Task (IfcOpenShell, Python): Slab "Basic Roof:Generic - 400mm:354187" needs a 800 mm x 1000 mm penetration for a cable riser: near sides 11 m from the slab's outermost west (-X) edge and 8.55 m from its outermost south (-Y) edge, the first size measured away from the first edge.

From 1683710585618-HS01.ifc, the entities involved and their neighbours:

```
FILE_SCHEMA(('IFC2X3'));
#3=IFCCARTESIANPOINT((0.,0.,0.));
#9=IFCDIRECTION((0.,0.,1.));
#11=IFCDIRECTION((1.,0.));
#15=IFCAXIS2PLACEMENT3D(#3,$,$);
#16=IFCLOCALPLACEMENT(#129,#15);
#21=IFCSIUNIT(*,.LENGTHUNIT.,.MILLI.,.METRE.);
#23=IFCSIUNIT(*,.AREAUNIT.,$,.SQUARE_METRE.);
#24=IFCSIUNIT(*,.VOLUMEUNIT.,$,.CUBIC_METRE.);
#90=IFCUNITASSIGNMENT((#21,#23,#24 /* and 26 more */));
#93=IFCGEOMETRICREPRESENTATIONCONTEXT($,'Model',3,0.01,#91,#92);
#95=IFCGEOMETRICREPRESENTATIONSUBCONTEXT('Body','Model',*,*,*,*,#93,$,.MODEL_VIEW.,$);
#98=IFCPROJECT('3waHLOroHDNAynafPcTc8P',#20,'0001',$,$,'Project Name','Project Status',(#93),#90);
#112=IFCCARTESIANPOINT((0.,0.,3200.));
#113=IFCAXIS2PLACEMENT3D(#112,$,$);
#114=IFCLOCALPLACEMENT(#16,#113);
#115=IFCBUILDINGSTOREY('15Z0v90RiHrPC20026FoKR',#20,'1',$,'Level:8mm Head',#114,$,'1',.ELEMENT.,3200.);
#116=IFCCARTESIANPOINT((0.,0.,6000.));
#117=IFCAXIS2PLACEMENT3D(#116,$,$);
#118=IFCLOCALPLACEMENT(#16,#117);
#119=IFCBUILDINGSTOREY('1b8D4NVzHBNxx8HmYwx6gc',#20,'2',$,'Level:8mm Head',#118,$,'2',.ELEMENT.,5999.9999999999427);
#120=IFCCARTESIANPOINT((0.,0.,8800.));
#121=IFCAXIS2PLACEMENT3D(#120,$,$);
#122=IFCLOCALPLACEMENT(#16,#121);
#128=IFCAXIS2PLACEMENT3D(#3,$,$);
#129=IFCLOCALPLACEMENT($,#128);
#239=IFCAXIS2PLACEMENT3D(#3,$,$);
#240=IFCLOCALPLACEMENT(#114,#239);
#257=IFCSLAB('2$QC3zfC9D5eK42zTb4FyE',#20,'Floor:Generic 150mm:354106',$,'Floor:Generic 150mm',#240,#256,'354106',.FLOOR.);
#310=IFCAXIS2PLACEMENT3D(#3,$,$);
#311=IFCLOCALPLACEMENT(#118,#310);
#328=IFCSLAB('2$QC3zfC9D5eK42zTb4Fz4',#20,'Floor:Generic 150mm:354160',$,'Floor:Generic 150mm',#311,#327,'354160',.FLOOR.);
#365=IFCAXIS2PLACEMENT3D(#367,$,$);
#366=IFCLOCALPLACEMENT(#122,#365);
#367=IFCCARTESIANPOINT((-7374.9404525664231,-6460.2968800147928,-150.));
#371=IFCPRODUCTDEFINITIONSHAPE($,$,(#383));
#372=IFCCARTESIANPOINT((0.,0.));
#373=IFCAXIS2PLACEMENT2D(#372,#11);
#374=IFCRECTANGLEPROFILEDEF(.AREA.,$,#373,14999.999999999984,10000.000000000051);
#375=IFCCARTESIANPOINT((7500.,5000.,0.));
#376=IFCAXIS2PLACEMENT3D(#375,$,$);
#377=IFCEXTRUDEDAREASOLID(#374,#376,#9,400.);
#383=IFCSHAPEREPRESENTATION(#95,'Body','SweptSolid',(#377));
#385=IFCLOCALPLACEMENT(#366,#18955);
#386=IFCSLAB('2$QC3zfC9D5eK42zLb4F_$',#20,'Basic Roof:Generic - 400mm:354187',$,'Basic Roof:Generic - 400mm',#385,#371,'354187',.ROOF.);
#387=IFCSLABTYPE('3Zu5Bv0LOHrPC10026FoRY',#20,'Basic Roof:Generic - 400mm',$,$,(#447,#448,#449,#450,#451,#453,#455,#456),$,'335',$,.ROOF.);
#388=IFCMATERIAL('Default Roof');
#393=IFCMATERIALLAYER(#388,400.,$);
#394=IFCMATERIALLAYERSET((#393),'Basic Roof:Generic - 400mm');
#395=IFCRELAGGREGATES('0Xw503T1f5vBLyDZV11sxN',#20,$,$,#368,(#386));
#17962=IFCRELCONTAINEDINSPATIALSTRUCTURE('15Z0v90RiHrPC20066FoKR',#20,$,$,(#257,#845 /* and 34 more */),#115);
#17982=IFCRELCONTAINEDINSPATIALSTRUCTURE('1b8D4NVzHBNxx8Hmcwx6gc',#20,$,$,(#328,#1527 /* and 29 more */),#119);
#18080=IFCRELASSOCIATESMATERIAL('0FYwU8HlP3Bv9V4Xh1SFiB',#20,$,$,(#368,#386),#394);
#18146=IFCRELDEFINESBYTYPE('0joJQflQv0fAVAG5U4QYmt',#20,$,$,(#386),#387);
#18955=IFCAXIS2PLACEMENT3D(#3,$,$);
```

```python
import numpy as np
import ifcopenshell
import ifcopenshell.api.feature
import ifcopenshell.api.geometry
import ifcopenshell.api.root
import ifcopenshell.geom
import ifcopenshell.util.placement
import ifcopenshell.util.representation
import ifcopenshell.util.shape
import ifcopenshell.util.unit

model = ifcopenshell.open("1683710585618-HS01.ifc")
unit_scale = ifcopenshell.util.unit.calculate_unit_scale(model)
settings = ifcopenshell.geom.settings()


def volume(element):
    """Net volume in cubic metres, openings subtracted."""
    shape = ifcopenshell.geom.create_shape(settings, element)
    return ifcopenshell.util.shape.get_volume(shape.geometry)


slab = model.by_id(386)
before = volume(slab)

# Extent in the slab's own axes, in metres. The edges named are its -X and -Y sides.
slab_shape = ifcopenshell.geom.create_shape(settings, slab)
vertices = ifcopenshell.util.shape.get_vertices(slab_shape.geometry)
x_min, y_min, bottom = vertices.min(axis=0)
top = vertices[:, 2].max()

opening = ifcopenshell.api.root.create_entity(model, ifc_class="IfcOpeningElement", name="Cable riser opening")
context = ifcopenshell.util.representation.get_context(model, "Model", "Body", "MODEL_VIEW")
width, depth = 0.8, 1
outline = [(0.0, 0.0), (width, 0.0), (width, depth), (0.0, depth), (0.0, 0.0)]
# Overshoot both faces by 50 mm so the cut is clean.
shape = ifcopenshell.api.geometry.add_slab_representation(
    model, context=context, depth=top - bottom + 0.1, polyline=outline
)
ifcopenshell.api.geometry.assign_representation(model, product=opening, representation=shape)

matrix = ifcopenshell.util.placement.get_local_placement(slab.ObjectPlacement)
matrix[:, 3] = matrix @ np.append(np.array([x_min + 11, y_min + 8.55, bottom - 0.05]) / unit_scale, 1.0)
ifcopenshell.api.geometry.edit_object_placement(model, product=opening, matrix=matrix, is_si=False)
ifcopenshell.api.feature.add_feature(model, feature=opening, element=slab)

after = volume(slab)

print(f"slab volume {before:.3f} -> {after:.3f} m3")

model.write("1683710585618-HS01_v2.ifc")
```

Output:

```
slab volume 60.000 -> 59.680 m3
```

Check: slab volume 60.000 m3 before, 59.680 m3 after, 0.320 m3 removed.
